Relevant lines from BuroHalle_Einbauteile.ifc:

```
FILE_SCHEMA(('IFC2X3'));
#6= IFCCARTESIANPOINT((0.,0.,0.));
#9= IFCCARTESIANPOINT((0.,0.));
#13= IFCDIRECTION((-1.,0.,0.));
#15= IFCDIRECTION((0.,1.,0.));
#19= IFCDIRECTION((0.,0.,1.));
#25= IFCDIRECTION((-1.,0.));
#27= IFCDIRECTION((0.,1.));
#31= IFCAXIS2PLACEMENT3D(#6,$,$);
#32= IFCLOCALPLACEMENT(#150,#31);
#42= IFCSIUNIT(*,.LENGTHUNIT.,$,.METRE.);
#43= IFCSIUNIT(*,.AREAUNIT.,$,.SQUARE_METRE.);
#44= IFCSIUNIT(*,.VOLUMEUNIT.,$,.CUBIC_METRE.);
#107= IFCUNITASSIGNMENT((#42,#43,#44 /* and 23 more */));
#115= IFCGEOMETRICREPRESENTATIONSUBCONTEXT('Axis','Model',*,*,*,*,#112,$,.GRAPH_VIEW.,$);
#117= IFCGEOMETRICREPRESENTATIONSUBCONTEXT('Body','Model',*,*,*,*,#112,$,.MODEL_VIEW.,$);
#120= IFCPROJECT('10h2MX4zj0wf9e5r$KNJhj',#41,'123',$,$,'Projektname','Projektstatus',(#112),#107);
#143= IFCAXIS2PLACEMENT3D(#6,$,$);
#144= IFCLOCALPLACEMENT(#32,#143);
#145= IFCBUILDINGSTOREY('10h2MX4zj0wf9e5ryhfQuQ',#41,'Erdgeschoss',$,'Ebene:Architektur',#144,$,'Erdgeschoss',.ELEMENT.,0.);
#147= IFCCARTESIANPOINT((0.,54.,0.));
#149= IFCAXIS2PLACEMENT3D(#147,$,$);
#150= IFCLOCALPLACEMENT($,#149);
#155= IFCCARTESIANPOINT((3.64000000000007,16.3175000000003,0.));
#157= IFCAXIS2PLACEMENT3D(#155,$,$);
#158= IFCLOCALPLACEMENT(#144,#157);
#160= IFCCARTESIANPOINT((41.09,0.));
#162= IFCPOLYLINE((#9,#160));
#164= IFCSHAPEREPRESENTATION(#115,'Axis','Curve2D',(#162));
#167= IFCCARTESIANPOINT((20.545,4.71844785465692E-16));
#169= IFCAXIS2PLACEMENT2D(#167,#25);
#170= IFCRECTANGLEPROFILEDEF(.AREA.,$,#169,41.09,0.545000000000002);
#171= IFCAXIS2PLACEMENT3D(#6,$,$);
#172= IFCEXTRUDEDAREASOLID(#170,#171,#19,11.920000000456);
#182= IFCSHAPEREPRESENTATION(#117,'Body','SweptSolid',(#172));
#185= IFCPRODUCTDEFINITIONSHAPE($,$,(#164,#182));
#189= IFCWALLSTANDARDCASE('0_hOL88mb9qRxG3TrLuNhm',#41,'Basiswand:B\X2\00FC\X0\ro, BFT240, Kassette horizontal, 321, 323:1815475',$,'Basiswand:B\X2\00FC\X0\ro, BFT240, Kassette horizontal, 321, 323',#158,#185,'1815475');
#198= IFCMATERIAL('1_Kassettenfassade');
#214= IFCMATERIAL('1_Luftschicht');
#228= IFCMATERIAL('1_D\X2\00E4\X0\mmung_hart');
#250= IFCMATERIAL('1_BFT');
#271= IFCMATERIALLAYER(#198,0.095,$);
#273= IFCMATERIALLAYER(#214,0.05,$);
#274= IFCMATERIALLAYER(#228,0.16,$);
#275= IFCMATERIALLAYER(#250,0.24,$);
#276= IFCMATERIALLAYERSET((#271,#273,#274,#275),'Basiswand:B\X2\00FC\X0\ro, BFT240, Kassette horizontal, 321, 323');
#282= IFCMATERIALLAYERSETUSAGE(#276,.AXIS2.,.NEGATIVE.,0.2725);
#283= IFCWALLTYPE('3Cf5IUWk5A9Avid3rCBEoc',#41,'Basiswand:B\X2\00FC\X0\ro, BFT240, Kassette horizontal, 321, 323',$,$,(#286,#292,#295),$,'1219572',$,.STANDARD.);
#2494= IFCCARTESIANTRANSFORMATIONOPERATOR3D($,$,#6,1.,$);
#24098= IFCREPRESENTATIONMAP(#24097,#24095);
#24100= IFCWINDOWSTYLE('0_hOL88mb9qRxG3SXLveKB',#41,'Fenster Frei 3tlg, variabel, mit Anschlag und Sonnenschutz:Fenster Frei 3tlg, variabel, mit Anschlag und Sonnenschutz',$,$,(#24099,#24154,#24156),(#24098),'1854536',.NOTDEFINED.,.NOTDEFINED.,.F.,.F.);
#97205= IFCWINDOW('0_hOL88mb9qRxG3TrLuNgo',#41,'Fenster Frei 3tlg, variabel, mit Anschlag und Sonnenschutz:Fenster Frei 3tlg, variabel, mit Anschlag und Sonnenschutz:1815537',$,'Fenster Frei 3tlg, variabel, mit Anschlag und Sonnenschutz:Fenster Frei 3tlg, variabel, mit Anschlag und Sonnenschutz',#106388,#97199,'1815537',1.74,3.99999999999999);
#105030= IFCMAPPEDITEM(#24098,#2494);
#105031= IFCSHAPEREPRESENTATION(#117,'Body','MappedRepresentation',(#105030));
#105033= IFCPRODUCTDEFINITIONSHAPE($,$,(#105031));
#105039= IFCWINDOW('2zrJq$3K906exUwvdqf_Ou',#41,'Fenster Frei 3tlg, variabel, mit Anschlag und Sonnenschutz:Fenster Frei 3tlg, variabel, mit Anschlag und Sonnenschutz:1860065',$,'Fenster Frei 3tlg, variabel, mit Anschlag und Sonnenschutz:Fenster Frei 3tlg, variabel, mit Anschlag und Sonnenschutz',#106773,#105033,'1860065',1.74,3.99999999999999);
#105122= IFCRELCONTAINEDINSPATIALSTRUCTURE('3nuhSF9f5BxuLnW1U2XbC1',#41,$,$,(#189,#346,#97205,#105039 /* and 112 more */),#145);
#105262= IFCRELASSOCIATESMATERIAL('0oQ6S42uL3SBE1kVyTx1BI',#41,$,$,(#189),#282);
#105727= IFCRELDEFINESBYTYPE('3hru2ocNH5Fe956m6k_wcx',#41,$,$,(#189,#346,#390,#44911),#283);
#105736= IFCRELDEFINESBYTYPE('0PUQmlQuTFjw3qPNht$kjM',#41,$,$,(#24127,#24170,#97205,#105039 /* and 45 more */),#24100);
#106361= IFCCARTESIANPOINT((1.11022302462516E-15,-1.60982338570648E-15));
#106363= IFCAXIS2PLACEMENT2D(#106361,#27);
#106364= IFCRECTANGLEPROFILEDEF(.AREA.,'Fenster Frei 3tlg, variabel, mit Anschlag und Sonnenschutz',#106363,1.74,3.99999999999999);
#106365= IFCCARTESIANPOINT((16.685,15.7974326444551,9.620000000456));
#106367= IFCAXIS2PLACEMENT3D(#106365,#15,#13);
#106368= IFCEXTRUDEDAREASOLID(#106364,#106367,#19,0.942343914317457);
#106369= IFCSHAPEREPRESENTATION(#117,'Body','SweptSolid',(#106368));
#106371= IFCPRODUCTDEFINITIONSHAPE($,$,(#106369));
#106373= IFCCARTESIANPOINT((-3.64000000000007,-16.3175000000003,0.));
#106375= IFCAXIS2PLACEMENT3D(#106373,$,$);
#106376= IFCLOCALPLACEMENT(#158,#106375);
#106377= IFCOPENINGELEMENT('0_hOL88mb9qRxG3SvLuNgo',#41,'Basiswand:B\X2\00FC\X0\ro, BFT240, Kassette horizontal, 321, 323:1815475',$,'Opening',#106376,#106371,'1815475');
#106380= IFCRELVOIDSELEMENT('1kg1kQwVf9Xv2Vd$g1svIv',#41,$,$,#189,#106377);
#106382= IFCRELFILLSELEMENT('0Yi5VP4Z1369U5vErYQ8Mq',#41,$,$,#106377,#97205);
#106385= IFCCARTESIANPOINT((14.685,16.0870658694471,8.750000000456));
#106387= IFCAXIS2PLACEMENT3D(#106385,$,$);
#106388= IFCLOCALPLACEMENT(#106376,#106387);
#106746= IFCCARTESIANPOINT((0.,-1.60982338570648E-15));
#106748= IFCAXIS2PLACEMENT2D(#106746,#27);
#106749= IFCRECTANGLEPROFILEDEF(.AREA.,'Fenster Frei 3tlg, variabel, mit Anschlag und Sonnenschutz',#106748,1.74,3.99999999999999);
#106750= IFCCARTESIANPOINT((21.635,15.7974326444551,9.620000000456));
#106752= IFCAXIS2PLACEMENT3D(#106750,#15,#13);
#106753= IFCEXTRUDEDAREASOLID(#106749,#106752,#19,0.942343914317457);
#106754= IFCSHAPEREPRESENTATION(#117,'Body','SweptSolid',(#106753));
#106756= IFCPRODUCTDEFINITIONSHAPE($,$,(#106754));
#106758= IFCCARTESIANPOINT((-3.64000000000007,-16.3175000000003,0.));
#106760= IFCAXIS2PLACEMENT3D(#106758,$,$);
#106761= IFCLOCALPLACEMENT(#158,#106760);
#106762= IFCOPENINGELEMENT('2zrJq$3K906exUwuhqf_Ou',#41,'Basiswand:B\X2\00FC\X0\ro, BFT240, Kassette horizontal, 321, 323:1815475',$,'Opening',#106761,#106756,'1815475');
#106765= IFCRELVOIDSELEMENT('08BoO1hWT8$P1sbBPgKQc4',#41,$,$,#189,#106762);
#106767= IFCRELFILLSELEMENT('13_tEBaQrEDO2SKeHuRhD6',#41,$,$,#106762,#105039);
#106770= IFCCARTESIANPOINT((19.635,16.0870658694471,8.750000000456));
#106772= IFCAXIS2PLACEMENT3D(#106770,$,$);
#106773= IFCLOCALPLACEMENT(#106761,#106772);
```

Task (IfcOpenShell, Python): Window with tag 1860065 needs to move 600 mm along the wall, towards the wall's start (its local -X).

```python
import ifcopenshell
import ifcopenshell.api.geometry
import ifcopenshell.util.placement

model = ifcopenshell.open("BuroHalle_Einbauteile.ifc")

window = model.by_guid("2zrJq$3K906exUwvdqf_Ou")
opening = window.FillsVoids[0].RelatingOpeningElement
wall = opening.VoidsElements[0].RelatingBuildingElement

wall_matrix = ifcopenshell.util.placement.get_local_placement(wall.ObjectPlacement)
shift = wall_matrix[:3, 0] * -0.6
before = ifcopenshell.util.placement.get_local_placement(window.ObjectPlacement)[:3, 3].copy()

# The window is placed relative to its opening, so it follows when the opening moves.
matrix = ifcopenshell.util.placement.get_local_placement(opening.ObjectPlacement)
matrix[:3, 3] += shift
ifcopenshell.api.geometry.edit_object_placement(
    model, product=opening, matrix=matrix, is_si=False, should_transform_children=True
)

after = ifcopenshell.util.placement.get_local_placement(window.ObjectPlacement)[:3, 3]
print("window moved by", (after - before).round(3) + 0.0)

model.write("BuroHalle_Einbauteile_edited.ifc")
```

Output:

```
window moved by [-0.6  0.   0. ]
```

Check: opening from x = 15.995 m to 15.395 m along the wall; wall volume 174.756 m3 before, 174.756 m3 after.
